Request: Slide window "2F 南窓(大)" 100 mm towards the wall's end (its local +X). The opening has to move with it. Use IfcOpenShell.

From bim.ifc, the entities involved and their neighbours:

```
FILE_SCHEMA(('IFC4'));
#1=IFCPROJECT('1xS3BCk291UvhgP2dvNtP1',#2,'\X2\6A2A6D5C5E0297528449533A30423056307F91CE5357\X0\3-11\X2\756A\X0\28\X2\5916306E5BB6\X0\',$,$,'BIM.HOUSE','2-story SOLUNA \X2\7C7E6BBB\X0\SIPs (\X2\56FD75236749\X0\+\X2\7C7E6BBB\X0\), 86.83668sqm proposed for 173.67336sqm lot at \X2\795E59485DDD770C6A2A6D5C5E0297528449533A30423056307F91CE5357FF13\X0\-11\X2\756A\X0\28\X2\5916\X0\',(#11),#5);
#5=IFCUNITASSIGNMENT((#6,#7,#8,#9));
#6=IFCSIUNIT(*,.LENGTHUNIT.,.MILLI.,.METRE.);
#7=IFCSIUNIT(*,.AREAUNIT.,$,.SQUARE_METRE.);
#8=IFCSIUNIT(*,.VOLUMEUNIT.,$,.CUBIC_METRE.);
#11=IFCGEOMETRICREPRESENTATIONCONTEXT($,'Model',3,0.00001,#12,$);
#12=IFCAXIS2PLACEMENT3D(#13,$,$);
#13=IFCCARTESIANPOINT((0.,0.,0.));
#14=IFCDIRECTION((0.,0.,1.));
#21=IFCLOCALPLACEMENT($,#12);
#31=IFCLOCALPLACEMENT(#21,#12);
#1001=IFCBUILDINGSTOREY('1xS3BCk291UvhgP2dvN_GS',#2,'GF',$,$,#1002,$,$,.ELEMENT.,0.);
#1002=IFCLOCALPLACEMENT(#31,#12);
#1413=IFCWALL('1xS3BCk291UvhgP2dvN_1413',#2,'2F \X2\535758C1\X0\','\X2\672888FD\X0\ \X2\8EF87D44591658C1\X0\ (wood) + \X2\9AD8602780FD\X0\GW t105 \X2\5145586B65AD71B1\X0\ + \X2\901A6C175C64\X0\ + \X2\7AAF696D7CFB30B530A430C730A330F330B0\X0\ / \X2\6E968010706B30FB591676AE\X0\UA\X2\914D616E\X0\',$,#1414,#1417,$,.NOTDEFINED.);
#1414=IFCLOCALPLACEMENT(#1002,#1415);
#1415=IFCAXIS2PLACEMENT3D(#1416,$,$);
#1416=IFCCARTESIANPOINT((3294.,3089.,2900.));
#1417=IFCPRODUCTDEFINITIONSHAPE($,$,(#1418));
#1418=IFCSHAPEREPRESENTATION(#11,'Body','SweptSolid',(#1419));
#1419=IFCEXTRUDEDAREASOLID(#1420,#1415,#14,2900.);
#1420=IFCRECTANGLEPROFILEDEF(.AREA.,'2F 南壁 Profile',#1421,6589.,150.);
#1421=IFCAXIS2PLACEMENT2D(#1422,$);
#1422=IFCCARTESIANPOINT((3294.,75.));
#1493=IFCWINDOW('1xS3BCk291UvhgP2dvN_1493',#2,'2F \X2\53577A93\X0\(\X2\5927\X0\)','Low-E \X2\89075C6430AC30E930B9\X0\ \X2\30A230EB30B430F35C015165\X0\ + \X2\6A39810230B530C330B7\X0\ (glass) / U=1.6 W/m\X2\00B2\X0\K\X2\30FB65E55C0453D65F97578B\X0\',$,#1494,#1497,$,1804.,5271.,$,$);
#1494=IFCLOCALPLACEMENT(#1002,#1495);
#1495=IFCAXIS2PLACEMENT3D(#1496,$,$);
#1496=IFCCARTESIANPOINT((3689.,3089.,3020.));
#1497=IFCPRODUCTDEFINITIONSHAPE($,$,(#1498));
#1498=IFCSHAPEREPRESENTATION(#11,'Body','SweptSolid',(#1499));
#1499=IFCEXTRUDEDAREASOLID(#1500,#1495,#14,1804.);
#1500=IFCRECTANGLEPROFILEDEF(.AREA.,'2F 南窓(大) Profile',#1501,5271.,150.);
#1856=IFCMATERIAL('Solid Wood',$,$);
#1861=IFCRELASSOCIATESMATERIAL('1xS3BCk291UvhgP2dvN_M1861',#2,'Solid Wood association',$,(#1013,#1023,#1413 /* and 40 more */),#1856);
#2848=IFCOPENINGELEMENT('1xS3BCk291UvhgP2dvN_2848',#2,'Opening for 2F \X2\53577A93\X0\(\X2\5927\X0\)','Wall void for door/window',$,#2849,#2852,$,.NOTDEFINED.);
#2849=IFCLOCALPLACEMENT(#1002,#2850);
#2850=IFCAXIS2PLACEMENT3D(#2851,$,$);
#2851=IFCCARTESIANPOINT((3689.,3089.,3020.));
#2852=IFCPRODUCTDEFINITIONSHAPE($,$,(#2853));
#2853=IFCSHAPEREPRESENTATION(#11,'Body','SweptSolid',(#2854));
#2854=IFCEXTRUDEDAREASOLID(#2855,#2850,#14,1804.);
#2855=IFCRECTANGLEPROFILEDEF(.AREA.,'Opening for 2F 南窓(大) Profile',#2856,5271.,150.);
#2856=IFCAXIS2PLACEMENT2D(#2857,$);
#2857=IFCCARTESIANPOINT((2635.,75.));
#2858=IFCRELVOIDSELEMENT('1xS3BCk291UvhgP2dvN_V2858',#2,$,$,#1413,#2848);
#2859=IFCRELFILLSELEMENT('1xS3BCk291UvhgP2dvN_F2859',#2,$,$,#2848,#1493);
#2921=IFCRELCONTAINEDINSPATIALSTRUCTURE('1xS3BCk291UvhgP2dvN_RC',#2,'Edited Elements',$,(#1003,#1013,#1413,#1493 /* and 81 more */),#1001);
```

```python
import ifcopenshell
import ifcopenshell.api.geometry
import ifcopenshell.util.placement
import ifcopenshell.util.unit

model = ifcopenshell.open("bim.ifc")
unit_scale = ifcopenshell.util.unit.calculate_unit_scale(model)

window = model.by_guid("1xS3BCk291UvhgP2dvN_1493")
opening = window.FillsVoids[0].RelatingOpeningElement
wall = opening.VoidsElements[0].RelatingBuildingElement

wall_matrix = ifcopenshell.util.placement.get_local_placement(wall.ObjectPlacement)
shift = wall_matrix[:3, 0] * 0.1 / unit_scale
before = ifcopenshell.util.placement.get_local_placement(window.ObjectPlacement)[:3, 3].copy()

# The window is not placed relative to its opening, so move both.
for product in (opening, window):
    matrix = ifcopenshell.util.placement.get_local_placement(product.ObjectPlacement)
    matrix[:3, 3] += shift
    ifcopenshell.api.geometry.edit_object_placement(model, product=product, matrix=matrix, is_si=False)

after = ifcopenshell.util.placement.get_local_placement(window.ObjectPlacement)[:3, 3]
print("window moved by", (after - before).round(3) + 0.0)

model.write("bim_rev.ifc")
```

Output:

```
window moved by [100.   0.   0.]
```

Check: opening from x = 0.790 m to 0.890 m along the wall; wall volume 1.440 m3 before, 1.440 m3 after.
